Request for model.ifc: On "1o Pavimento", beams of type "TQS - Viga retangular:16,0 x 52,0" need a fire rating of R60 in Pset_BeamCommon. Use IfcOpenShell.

First a look at what the model holds.

```python
import ifcopenshell
import ifcopenshell.util.element

model = ifcopenshell.open("model.ifc")
print(model.schema)
storey = next(s for s in model.by_type("IfcBuildingStorey") if s.Name == "1o Pavimento")
beams = [e for e in ifcopenshell.util.element.get_decomposition(storey) if e.is_a("IfcBeam")]
seen = {}
for e in beams:
    element_type = ifcopenshell.util.element.get_type(e)
    key = (element_type.Name if element_type != e and element_type else None, ifcopenshell.util.element.get_pset(e, "Pset_BeamCommon", "FireRating"))
    seen[key] = seen.get(key, 0) + 1
for (name, value), count in sorted(seen.items(), key=str):
    print(count, "x", name, "|", value)
```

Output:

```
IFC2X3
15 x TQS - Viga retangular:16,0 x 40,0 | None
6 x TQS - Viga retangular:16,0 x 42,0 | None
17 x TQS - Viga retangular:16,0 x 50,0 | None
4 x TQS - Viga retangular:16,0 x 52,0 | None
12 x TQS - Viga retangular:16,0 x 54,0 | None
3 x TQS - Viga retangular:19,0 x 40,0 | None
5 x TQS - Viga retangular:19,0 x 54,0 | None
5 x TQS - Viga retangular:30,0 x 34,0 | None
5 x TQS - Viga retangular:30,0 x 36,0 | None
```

```python
import ifcopenshell
import ifcopenshell.api.pset
import ifcopenshell.util.element

model = ifcopenshell.open("model.ifc")

storey = next(s for s in model.by_type("IfcBuildingStorey") if s.Name == "1o Pavimento")
beams = [e for e in ifcopenshell.util.element.get_decomposition(storey) if e.is_a("IfcBeam")]

count = 0
for e in beams:
    element_type = ifcopenshell.util.element.get_type(e)
    if element_type in (None, e) or element_type.Name != "TQS - Viga retangular:16,0 x 52,0":
        continue
    # add_pset returns the element's existing set when there is one.
    pset = ifcopenshell.api.pset.add_pset(model, product=e, name="Pset_BeamCommon")
    ifcopenshell.api.pset.edit_pset(model, pset=pset, properties={"FireRating": "R60"})
    count += 1

print(count, "beams updated")

model.write("model_edited.ifc")
```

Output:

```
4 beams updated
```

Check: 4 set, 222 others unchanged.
